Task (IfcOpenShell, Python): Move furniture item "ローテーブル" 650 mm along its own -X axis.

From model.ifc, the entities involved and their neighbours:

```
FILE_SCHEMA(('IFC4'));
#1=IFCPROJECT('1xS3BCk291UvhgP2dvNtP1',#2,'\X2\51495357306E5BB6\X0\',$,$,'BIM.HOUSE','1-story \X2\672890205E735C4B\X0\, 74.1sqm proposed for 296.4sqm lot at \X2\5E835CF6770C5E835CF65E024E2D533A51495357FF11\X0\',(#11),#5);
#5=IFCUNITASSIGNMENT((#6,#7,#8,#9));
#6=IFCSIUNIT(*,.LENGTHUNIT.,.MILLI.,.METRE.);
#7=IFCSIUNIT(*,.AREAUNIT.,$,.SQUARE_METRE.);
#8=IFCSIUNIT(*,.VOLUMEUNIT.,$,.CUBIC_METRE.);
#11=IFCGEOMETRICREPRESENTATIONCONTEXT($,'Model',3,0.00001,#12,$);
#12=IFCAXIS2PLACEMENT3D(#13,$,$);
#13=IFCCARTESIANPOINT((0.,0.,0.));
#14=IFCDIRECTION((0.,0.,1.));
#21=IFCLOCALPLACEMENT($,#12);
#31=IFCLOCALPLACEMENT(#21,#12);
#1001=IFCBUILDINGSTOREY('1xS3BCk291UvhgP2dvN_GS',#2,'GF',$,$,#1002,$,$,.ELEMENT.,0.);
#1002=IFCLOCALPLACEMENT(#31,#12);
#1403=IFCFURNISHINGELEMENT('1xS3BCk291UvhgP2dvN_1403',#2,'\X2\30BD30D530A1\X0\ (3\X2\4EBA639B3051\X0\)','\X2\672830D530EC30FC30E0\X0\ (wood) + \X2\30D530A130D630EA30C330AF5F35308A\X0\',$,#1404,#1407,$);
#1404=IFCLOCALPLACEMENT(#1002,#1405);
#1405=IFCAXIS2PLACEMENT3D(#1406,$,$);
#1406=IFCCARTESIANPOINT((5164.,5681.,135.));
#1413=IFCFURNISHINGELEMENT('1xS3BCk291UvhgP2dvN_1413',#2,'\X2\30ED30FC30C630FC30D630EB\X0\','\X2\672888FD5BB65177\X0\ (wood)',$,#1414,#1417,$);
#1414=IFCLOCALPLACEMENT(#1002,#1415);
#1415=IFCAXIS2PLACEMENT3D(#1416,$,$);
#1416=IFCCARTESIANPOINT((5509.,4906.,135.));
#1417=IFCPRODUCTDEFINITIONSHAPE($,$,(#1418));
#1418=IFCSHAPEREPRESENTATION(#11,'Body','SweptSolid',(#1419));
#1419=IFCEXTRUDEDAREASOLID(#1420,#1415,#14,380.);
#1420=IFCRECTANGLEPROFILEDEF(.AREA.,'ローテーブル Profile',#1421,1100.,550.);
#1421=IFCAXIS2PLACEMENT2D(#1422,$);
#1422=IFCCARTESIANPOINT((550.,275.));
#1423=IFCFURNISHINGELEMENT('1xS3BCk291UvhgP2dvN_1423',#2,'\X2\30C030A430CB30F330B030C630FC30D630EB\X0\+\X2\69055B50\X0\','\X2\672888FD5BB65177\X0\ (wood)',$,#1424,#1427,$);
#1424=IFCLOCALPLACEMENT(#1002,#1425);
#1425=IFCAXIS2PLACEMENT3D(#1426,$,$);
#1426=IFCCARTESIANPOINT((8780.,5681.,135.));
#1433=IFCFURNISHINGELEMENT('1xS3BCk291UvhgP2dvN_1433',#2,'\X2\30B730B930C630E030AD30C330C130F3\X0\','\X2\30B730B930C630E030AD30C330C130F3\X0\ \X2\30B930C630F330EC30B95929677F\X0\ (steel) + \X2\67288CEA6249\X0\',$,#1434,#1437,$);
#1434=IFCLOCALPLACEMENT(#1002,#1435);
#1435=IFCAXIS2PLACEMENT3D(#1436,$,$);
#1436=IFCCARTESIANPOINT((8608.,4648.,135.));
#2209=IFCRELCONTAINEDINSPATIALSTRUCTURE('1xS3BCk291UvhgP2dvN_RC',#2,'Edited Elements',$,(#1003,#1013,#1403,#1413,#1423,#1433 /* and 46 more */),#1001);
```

```python
import ifcopenshell
import ifcopenshell.api.geometry
import ifcopenshell.util.placement
import ifcopenshell.util.unit

model = ifcopenshell.open("model.ifc")
unit_scale = ifcopenshell.util.unit.calculate_unit_scale(model)

item = model.by_guid("1xS3BCk291UvhgP2dvN_1413")
matrix = ifcopenshell.util.placement.get_local_placement(item.ObjectPlacement)
matrix[:3, 3] -= matrix[:3, 0] * 0.65 / unit_scale
ifcopenshell.api.geometry.edit_object_placement(model, product=item, matrix=matrix, is_si=False)

print(ifcopenshell.util.placement.get_local_placement(item.ObjectPlacement).round(3) + 0.0)

model.write("model_updated.ifc")
```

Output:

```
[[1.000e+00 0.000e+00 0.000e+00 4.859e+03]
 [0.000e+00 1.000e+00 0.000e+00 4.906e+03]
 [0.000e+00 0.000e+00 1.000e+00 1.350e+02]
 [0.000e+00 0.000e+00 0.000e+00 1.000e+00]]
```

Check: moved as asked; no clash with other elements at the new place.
